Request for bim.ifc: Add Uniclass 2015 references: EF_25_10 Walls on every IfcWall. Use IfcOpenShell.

First a look at what the model holds.

```python
import ifcopenshell

model = ifcopenshell.open("bim.ifc")
print(model.schema)
print("classifications:", [c.Name for c in model.by_type("IfcClassification")])
for ifc_class in ("IfcDoor", "IfcRoof", "IfcStair", "IfcWall", "IfcWindow"):
    print(ifc_class, len(model.by_type(ifc_class)))
```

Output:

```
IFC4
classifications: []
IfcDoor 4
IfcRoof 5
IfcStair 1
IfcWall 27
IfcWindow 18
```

```python
import ifcopenshell
import ifcopenshell.api.classification

model = ifcopenshell.open("bim.ifc")

system = ifcopenshell.api.classification.add_classification(model, classification="Uniclass 2015")

codes = {
    "IfcWall": ("EF_25_10", "Walls"),
}
for ifc_class, (code, name) in codes.items():
    products = model.by_type(ifc_class)
    ifcopenshell.api.classification.add_reference(
        model, products=products, classification=system, identification=code, name=name
    )
    print(code, len(products))

model.write("bim_rev.ifc")
```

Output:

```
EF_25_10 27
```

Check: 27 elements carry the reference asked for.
